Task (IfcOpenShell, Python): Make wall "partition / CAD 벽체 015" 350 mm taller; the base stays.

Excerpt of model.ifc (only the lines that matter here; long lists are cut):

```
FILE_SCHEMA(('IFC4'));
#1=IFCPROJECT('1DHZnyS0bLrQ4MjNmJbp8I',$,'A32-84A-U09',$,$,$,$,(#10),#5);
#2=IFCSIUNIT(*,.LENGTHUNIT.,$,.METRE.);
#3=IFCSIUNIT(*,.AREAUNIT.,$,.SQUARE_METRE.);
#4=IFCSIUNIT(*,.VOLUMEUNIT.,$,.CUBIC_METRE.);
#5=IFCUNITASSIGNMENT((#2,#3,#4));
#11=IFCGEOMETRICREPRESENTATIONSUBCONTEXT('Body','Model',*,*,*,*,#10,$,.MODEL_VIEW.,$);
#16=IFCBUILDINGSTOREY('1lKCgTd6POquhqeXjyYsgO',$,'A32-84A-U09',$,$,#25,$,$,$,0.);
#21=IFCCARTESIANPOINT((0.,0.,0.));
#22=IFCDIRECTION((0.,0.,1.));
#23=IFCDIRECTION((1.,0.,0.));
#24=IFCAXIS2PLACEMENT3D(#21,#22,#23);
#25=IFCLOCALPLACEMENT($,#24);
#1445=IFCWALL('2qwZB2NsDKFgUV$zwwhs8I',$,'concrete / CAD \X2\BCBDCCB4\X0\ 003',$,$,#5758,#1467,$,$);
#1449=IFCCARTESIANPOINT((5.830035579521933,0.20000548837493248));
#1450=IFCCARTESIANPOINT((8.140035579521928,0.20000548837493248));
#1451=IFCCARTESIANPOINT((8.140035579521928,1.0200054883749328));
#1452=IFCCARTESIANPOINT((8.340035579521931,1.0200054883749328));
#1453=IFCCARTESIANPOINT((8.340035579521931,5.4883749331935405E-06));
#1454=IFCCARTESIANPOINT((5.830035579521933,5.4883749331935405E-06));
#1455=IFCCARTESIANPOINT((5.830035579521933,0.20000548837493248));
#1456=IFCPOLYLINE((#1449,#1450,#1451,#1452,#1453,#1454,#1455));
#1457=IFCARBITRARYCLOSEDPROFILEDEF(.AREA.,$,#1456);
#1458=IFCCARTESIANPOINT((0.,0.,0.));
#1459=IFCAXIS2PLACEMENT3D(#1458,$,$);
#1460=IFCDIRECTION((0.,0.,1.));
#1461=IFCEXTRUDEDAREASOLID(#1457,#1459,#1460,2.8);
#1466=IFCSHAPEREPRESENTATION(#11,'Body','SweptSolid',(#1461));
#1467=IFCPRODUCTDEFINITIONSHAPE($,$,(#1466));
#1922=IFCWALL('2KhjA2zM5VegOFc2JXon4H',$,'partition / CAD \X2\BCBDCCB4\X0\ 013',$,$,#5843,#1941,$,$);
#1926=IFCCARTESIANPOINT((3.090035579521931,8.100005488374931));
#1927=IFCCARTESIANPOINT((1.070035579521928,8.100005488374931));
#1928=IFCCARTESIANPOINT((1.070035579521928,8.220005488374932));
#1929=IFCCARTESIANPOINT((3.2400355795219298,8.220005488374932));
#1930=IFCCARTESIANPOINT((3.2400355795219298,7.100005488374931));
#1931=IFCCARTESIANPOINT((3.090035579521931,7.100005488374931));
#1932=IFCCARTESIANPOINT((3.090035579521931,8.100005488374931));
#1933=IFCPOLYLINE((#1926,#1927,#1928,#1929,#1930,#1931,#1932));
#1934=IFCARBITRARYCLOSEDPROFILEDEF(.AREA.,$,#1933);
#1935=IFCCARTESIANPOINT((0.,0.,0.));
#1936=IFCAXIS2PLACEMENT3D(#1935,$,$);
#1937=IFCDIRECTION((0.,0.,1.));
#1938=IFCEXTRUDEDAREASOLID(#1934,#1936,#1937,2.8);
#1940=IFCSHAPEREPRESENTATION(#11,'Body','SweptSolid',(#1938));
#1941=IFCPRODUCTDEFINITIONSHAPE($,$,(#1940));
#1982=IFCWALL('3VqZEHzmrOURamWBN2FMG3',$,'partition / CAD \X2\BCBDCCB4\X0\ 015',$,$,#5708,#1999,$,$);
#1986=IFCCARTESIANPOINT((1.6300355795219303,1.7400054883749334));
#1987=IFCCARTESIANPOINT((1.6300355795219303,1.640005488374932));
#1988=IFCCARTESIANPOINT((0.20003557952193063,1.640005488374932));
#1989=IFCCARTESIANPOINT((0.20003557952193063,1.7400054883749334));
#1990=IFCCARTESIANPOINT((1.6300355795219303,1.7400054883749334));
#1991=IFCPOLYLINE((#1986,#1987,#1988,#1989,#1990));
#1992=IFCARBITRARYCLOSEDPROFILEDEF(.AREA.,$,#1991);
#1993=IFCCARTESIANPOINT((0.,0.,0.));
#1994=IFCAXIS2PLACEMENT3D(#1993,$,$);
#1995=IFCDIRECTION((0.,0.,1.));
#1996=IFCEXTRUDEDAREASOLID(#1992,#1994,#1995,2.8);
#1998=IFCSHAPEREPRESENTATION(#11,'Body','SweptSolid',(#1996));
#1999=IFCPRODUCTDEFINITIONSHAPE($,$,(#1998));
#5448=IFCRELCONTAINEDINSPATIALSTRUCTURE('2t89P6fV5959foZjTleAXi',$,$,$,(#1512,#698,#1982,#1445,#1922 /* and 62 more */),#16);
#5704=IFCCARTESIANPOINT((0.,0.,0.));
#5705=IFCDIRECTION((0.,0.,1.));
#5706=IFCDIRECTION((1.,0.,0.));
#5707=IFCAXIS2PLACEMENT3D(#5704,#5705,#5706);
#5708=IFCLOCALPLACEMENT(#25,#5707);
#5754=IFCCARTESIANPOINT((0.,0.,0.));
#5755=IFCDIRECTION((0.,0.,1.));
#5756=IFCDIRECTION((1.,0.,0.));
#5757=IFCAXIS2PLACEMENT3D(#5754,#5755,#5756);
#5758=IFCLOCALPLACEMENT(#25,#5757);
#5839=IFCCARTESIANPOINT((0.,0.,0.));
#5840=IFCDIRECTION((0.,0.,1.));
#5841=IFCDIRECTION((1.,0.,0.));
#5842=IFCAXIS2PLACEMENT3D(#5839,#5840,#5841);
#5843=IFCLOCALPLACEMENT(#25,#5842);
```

```python
import ifcopenshell
import ifcopenshell.geom
import ifcopenshell.util.representation
import ifcopenshell.util.shape
import ifcopenshell.util.unit

model = ifcopenshell.open("model.ifc")
unit_scale = ifcopenshell.util.unit.calculate_unit_scale(model)
settings = ifcopenshell.geom.settings()


def volume(element):
    """Net volume in cubic metres, openings subtracted."""
    shape = ifcopenshell.geom.create_shape(settings, element)
    return ifcopenshell.util.shape.get_volume(shape.geometry)


wall = model.by_id(1982)
before = volume(wall)

body = ifcopenshell.util.representation.get_representation(wall, "Model", "Body")
solid = body.Items[0]
old_height = solid.Depth
solid.Depth += 0.35 / unit_scale
after = volume(wall)

print(f"height {old_height:g} -> {solid.Depth:g}, volume {before:.3f} -> {after:.3f} m3")

model.write("model_v2.ifc")
```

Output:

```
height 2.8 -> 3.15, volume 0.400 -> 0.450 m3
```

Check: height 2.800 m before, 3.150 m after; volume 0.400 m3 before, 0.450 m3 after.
